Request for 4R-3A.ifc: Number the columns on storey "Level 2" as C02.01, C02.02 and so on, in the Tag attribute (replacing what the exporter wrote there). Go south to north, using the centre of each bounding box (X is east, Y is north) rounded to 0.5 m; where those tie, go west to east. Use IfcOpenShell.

First a look at what the model holds.

```python
import ifcopenshell
import ifcopenshell.util.element
import ifcopenshell.util.placement

model = ifcopenshell.open("4R-3A.ifc")
print(model.schema)
storey = next(s for s in model.by_type("IfcBuildingStorey") if s.Name == "Level 2")
columns = [e for e in ifcopenshell.util.element.get_decomposition(storey) if e.is_a("IfcColumn")]
for e in sorted(columns, key=lambda e: e.id()):
    origin = ifcopenshell.util.placement.get_local_placement(e.ObjectPlacement)[:3, 3]
    print(e.id(), e.Tag, e.Name, origin.round(2) + 0.0, sep=" | ")
```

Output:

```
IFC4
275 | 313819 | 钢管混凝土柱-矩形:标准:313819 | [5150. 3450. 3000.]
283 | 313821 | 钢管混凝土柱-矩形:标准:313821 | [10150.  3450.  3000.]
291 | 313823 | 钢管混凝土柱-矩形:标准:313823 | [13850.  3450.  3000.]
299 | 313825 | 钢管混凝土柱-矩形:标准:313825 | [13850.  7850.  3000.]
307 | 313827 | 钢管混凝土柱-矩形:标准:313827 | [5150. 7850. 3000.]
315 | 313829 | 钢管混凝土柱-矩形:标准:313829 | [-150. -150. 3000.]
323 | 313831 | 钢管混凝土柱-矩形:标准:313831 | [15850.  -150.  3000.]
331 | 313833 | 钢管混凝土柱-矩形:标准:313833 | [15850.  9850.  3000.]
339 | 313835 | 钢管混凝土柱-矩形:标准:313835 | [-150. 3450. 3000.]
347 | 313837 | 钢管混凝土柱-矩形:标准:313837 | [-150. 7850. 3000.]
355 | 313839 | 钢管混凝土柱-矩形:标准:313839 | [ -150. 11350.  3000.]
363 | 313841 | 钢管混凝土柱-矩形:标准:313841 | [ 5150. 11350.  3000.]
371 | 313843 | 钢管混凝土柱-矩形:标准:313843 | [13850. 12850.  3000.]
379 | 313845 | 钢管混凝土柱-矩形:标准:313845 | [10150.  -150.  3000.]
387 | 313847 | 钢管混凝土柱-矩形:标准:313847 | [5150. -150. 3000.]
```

```python
import ifcopenshell
import ifcopenshell.geom
import ifcopenshell.util.element
import ifcopenshell.util.shape

model = ifcopenshell.open("4R-3A.ifc")
settings = ifcopenshell.geom.settings()
settings.set("use-world-coords", True)


def centre(element):
    shape = ifcopenshell.geom.create_shape(settings, element)
    return ifcopenshell.util.shape.get_bbox_centroid(shape.geometry)


storey = next(s for s in model.by_type("IfcBuildingStorey") if s.Name == "Level 2")
columns = [e for e in ifcopenshell.util.element.get_decomposition(storey) if e.is_a("IfcColumn")]

# Insertion points can sit at a corner or the storey origin, so sort by the geometry (in metres).
centres = {e: centre(e) for e in columns}
columns.sort(key=lambda e: (round(centres[e][1] / 0.5), centres[e][0]))

for i, e in enumerate(columns, start=1):
    number = f"C02.{i:02d}"
    e.Tag = number
    print(e.id(), number)

model.write("4R-3A_rev.ifc")
```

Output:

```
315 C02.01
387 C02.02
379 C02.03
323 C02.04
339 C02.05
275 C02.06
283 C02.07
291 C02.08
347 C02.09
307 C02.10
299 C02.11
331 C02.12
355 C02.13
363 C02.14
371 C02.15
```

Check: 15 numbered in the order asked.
